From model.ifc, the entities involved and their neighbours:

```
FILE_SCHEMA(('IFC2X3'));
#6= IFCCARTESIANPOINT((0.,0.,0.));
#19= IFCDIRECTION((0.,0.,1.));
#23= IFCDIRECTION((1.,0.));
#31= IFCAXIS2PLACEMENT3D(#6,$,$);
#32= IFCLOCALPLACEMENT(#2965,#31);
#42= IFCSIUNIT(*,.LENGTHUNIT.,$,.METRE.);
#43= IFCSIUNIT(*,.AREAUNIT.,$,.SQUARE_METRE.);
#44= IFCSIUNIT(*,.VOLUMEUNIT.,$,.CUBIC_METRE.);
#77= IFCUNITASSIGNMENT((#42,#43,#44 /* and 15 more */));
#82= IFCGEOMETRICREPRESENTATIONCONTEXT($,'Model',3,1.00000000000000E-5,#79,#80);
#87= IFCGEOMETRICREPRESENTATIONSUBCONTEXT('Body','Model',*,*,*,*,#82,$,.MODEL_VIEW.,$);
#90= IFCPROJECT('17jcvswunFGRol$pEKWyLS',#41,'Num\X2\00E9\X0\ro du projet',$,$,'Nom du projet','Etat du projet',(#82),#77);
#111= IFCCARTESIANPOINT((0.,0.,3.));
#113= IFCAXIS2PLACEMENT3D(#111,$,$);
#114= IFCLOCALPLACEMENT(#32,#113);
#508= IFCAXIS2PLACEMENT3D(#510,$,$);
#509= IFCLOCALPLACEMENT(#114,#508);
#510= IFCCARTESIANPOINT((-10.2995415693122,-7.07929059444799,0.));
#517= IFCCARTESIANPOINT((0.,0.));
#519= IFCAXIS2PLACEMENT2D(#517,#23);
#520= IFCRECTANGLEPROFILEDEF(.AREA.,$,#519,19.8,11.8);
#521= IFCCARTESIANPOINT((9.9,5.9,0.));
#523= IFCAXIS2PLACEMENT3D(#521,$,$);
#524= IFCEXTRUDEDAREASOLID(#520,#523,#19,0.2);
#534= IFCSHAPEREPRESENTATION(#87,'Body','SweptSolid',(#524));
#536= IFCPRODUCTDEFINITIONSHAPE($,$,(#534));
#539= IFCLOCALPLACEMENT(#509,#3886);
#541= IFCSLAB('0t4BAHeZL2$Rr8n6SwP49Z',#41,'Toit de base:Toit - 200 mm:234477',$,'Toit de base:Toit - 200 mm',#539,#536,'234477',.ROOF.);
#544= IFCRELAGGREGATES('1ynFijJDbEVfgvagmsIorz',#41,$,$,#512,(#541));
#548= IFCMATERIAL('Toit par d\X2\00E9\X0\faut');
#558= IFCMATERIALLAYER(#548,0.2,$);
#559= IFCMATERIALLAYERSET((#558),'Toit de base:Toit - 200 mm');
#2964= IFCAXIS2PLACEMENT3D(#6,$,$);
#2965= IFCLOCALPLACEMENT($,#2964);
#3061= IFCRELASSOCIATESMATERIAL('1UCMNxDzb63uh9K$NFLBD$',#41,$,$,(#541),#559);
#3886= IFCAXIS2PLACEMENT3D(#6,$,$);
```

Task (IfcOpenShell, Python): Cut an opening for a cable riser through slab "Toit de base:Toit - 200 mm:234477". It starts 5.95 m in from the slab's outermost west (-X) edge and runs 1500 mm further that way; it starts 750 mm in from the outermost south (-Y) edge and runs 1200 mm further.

```python
import numpy as np
import ifcopenshell
import ifcopenshell.api.feature
import ifcopenshell.api.geometry
import ifcopenshell.api.root
import ifcopenshell.geom
import ifcopenshell.util.placement
import ifcopenshell.util.representation
import ifcopenshell.util.shape
import ifcopenshell.util.unit

model = ifcopenshell.open("model.ifc")
unit_scale = ifcopenshell.util.unit.calculate_unit_scale(model)
settings = ifcopenshell.geom.settings()


def volume(element):
    """Net volume in cubic metres, openings subtracted."""
    shape = ifcopenshell.geom.create_shape(settings, element)
    return ifcopenshell.util.shape.get_volume(shape.geometry)


slab = model.by_guid("0t4BAHeZL2$Rr8n6SwP49Z")
before = volume(slab)

# Extent in the slab's own axes, in metres. The edges named are its -X and -Y sides.
slab_shape = ifcopenshell.geom.create_shape(settings, slab)
vertices = ifcopenshell.util.shape.get_vertices(slab_shape.geometry)
x_min, y_min, bottom = vertices.min(axis=0)
top = vertices[:, 2].max()

opening = ifcopenshell.api.root.create_entity(model, ifc_class="IfcOpeningElement", name="Cable riser opening")
context = ifcopenshell.util.representation.get_context(model, "Model", "Body", "MODEL_VIEW")
width, depth = 1.5, 1.2
outline = [(0.0, 0.0), (width, 0.0), (width, depth), (0.0, depth), (0.0, 0.0)]
# Overshoot both faces by 50 mm so the cut is clean.
shape = ifcopenshell.api.geometry.add_slab_representation(
    model, context=context, depth=top - bottom + 0.1, polyline=outline
)
ifcopenshell.api.geometry.assign_representation(model, product=opening, representation=shape)

matrix = ifcopenshell.util.placement.get_local_placement(slab.ObjectPlacement)
matrix[:, 3] = matrix @ np.append(np.array([x_min + 5.95, y_min + 0.75, bottom - 0.05]) / unit_scale, 1.0)
ifcopenshell.api.geometry.edit_object_placement(model, product=opening, matrix=matrix, is_si=False)
ifcopenshell.api.feature.add_feature(model, feature=opening, element=slab)

after = volume(slab)

print(f"slab volume {before:.3f} -> {after:.3f} m3")

model.write("model_edited.ifc")
```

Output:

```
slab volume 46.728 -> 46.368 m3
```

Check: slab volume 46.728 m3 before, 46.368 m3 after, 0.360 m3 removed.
